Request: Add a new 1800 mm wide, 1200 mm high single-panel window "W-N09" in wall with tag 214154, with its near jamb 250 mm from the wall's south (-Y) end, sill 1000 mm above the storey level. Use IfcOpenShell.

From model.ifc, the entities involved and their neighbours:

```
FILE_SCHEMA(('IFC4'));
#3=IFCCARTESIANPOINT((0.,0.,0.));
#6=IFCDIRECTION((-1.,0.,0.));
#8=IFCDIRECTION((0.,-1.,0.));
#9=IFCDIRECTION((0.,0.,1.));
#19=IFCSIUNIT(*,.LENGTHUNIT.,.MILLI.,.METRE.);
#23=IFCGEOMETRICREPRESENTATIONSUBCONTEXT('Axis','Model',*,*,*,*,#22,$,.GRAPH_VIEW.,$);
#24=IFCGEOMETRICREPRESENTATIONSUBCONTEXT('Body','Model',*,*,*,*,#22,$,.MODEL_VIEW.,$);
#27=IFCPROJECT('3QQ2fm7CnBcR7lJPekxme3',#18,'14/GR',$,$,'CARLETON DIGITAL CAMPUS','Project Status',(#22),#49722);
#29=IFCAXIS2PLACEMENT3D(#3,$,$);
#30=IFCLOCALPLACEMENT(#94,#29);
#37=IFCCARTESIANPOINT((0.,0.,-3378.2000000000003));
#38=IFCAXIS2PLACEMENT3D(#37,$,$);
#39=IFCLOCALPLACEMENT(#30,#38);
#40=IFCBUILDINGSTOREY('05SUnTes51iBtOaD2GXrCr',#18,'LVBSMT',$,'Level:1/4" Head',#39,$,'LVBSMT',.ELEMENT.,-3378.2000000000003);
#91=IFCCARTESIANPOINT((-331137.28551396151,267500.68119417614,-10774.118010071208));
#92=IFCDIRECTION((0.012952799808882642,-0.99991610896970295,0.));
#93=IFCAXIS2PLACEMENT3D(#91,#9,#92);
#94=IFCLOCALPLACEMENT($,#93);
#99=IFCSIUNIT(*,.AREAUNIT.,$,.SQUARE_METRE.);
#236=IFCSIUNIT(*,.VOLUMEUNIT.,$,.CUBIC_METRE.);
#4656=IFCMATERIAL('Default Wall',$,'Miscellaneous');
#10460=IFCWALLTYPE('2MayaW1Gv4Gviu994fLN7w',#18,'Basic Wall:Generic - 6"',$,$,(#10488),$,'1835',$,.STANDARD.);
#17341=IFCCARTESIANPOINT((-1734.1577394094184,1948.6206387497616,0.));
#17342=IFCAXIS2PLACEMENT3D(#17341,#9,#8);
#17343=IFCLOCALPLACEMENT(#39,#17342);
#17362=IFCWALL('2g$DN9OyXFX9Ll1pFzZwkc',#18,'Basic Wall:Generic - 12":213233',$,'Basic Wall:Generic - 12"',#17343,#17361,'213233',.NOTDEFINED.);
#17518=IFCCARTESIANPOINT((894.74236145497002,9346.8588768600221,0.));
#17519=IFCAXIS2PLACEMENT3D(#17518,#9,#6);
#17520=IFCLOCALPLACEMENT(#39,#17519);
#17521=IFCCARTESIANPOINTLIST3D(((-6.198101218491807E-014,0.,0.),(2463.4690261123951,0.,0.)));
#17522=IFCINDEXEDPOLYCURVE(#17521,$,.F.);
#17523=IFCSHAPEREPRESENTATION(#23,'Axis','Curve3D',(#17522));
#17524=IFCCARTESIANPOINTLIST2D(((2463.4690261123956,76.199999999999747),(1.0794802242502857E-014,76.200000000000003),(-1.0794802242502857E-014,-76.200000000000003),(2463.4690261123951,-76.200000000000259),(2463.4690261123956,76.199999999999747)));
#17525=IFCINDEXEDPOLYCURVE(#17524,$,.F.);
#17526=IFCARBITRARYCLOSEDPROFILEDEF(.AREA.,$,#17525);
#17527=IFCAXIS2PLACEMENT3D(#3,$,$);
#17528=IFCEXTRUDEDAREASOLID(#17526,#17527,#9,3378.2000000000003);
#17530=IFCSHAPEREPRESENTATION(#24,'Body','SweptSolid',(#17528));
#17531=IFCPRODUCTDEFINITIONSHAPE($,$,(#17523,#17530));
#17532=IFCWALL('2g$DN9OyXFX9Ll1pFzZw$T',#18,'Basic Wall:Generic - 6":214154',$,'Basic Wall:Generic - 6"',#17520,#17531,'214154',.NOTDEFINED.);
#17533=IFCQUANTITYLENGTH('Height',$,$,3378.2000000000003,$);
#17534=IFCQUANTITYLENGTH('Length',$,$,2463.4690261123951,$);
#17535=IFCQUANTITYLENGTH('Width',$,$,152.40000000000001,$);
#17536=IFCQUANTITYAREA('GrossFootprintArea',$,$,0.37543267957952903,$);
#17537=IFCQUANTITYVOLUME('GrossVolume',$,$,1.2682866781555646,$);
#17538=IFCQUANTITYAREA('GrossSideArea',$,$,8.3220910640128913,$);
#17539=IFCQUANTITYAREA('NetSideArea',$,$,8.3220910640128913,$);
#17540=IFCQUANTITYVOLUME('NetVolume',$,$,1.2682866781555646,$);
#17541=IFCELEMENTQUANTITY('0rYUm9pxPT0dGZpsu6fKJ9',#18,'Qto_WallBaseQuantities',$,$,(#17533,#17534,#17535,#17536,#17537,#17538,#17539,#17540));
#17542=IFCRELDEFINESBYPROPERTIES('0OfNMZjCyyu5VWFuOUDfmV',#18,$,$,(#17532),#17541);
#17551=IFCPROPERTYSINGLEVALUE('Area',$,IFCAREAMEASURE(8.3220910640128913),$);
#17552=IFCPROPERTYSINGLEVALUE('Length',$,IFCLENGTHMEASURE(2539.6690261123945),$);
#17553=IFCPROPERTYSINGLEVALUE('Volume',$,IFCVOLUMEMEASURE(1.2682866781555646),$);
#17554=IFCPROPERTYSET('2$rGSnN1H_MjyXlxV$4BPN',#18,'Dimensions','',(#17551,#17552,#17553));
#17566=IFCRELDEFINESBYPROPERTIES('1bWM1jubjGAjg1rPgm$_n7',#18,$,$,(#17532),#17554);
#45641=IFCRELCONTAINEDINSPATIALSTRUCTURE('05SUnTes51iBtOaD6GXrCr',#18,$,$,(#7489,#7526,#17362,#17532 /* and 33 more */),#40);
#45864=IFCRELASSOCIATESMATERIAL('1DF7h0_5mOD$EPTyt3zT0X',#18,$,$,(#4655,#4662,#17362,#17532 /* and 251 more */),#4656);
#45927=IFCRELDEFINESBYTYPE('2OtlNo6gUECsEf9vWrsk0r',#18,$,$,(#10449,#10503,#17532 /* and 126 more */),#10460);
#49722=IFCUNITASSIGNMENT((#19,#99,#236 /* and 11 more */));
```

```python
import numpy as np
import ifcopenshell
import ifcopenshell.api.feature
import ifcopenshell.api.geometry
import ifcopenshell.api.pset
import ifcopenshell.api.root
import ifcopenshell.api.spatial
import ifcopenshell.geom
import ifcopenshell.util.element
import ifcopenshell.util.placement
import ifcopenshell.util.representation
import ifcopenshell.util.shape
import ifcopenshell.util.unit

model = ifcopenshell.open("model.ifc")
unit_scale = ifcopenshell.util.unit.calculate_unit_scale(model)
area_scale = ifcopenshell.util.unit.calculate_unit_scale(model, "AREAUNIT")
volume_scale = ifcopenshell.util.unit.calculate_unit_scale(model, "VOLUMEUNIT")
settings = ifcopenshell.geom.settings()


def volume(element):
    """Net volume in cubic metres, openings subtracted."""
    shape = ifcopenshell.geom.create_shape(settings, element)
    return ifcopenshell.util.shape.get_volume(shape.geometry)


wall = model.by_guid("2g$DN9OyXFX9Ll1pFzZw$T")
storey = ifcopenshell.util.element.get_container(wall, ifc_class="IfcBuildingStorey")
context = ifcopenshell.util.representation.get_context(model, "Model", "Body", "MODEL_VIEW")
before = volume(wall)

width, height, from_end, sill = 1.8, 1.2, 0.25, 1  # metres

# The wall runs along its own X axis, and the end named is its -X end.
wall_shape = ifcopenshell.geom.create_shape(settings, wall)
x, y, z = ifcopenshell.util.shape.get_vertices(wall_shape.geometry).T
start = x.min() + from_end
face, thickness = float(y.min()), float(y.max() - y.min())
wall_matrix = ifcopenshell.util.placement.get_local_placement(wall.ObjectPlacement)
level = ifcopenshell.util.placement.get_local_placement(storey.ObjectPlacement)[2, 3]


def in_wall(x, y):
    """Placement at x, y metres in the wall's axes, at sill height."""
    matrix = wall_matrix.copy()
    matrix[:, 3] = wall_matrix @ np.array([x / unit_scale, y / unit_scale, 0.0, 1.0])
    matrix[2, 3] = level + sill / unit_scale
    return matrix


# Opening: a box that overshoots both wall faces by 50 mm.
opening = ifcopenshell.api.root.create_entity(model, ifc_class="IfcOpeningElement", predefined_type="OPENING")
box = ifcopenshell.api.geometry.add_wall_representation(
    model, context=context, length=width, height=height, thickness=thickness + 0.1
)
ifcopenshell.api.geometry.assign_representation(model, product=opening, representation=box)
ifcopenshell.api.geometry.edit_object_placement(model, product=opening, matrix=in_wall(start, face - 0.05), is_si=False)
ifcopenshell.api.feature.add_feature(model, feature=opening, element=wall)

window = ifcopenshell.api.root.create_entity(model, ifc_class="IfcWindow", name="W-N09", predefined_type="WINDOW")
window.OverallWidth, window.OverallHeight = width / unit_scale, height / unit_scale
window.PartitioningType = "SINGLE_PANEL"
body = ifcopenshell.api.geometry.add_window_representation(
    model,
    context=context,
    overall_width=window.OverallWidth,
    overall_height=window.OverallHeight,
    partition_type="SINGLE_PANEL",
)
ifcopenshell.api.geometry.assign_representation(model, product=window, representation=body)
ifcopenshell.api.spatial.assign_container(model, products=[window], relating_structure=storey)
ifcopenshell.api.feature.add_filling(model, opening=opening, element=window)

# Centre the window in the wall's thickness.
ifcopenshell.api.geometry.edit_object_placement(model, product=window, matrix=in_wall(start, face), is_si=False)
window_shape = ifcopenshell.geom.create_shape(settings, window)
depth = ifcopenshell.util.shape.get_vertices(window_shape.geometry)[:, 1]
offset = face + thickness / 2 - (depth.min() + depth.max()) / 2
ifcopenshell.api.geometry.edit_object_placement(model, product=window, matrix=in_wall(start, offset), is_si=False)

after = volume(wall)

# Update the wall's stored quantities.
qto = model.by_id(ifcopenshell.util.element.get_pset(wall, "Qto_WallBaseQuantities", should_inherit=False)["id"])
ifcopenshell.api.pset.edit_qto(model, qto=qto, properties={
    "NetSideArea": after / thickness / area_scale,
    "NetVolume": after / volume_scale,
})
pset = model.by_id(ifcopenshell.util.element.get_pset(wall, "Dimensions", should_inherit=False)["id"])
ifcopenshell.api.pset.edit_pset(model, pset=pset, properties={
    "Area": model.create_entity("IfcAreaMeasure", after / thickness / area_scale),
    "Volume": model.create_entity("IfcVolumeMeasure", after / volume_scale),
})

print(f"wall volume {before:.3f} -> {after:.3f} m3")

model.write("model_v2.ifc")
```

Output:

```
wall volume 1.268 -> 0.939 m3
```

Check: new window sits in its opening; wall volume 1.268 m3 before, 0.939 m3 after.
